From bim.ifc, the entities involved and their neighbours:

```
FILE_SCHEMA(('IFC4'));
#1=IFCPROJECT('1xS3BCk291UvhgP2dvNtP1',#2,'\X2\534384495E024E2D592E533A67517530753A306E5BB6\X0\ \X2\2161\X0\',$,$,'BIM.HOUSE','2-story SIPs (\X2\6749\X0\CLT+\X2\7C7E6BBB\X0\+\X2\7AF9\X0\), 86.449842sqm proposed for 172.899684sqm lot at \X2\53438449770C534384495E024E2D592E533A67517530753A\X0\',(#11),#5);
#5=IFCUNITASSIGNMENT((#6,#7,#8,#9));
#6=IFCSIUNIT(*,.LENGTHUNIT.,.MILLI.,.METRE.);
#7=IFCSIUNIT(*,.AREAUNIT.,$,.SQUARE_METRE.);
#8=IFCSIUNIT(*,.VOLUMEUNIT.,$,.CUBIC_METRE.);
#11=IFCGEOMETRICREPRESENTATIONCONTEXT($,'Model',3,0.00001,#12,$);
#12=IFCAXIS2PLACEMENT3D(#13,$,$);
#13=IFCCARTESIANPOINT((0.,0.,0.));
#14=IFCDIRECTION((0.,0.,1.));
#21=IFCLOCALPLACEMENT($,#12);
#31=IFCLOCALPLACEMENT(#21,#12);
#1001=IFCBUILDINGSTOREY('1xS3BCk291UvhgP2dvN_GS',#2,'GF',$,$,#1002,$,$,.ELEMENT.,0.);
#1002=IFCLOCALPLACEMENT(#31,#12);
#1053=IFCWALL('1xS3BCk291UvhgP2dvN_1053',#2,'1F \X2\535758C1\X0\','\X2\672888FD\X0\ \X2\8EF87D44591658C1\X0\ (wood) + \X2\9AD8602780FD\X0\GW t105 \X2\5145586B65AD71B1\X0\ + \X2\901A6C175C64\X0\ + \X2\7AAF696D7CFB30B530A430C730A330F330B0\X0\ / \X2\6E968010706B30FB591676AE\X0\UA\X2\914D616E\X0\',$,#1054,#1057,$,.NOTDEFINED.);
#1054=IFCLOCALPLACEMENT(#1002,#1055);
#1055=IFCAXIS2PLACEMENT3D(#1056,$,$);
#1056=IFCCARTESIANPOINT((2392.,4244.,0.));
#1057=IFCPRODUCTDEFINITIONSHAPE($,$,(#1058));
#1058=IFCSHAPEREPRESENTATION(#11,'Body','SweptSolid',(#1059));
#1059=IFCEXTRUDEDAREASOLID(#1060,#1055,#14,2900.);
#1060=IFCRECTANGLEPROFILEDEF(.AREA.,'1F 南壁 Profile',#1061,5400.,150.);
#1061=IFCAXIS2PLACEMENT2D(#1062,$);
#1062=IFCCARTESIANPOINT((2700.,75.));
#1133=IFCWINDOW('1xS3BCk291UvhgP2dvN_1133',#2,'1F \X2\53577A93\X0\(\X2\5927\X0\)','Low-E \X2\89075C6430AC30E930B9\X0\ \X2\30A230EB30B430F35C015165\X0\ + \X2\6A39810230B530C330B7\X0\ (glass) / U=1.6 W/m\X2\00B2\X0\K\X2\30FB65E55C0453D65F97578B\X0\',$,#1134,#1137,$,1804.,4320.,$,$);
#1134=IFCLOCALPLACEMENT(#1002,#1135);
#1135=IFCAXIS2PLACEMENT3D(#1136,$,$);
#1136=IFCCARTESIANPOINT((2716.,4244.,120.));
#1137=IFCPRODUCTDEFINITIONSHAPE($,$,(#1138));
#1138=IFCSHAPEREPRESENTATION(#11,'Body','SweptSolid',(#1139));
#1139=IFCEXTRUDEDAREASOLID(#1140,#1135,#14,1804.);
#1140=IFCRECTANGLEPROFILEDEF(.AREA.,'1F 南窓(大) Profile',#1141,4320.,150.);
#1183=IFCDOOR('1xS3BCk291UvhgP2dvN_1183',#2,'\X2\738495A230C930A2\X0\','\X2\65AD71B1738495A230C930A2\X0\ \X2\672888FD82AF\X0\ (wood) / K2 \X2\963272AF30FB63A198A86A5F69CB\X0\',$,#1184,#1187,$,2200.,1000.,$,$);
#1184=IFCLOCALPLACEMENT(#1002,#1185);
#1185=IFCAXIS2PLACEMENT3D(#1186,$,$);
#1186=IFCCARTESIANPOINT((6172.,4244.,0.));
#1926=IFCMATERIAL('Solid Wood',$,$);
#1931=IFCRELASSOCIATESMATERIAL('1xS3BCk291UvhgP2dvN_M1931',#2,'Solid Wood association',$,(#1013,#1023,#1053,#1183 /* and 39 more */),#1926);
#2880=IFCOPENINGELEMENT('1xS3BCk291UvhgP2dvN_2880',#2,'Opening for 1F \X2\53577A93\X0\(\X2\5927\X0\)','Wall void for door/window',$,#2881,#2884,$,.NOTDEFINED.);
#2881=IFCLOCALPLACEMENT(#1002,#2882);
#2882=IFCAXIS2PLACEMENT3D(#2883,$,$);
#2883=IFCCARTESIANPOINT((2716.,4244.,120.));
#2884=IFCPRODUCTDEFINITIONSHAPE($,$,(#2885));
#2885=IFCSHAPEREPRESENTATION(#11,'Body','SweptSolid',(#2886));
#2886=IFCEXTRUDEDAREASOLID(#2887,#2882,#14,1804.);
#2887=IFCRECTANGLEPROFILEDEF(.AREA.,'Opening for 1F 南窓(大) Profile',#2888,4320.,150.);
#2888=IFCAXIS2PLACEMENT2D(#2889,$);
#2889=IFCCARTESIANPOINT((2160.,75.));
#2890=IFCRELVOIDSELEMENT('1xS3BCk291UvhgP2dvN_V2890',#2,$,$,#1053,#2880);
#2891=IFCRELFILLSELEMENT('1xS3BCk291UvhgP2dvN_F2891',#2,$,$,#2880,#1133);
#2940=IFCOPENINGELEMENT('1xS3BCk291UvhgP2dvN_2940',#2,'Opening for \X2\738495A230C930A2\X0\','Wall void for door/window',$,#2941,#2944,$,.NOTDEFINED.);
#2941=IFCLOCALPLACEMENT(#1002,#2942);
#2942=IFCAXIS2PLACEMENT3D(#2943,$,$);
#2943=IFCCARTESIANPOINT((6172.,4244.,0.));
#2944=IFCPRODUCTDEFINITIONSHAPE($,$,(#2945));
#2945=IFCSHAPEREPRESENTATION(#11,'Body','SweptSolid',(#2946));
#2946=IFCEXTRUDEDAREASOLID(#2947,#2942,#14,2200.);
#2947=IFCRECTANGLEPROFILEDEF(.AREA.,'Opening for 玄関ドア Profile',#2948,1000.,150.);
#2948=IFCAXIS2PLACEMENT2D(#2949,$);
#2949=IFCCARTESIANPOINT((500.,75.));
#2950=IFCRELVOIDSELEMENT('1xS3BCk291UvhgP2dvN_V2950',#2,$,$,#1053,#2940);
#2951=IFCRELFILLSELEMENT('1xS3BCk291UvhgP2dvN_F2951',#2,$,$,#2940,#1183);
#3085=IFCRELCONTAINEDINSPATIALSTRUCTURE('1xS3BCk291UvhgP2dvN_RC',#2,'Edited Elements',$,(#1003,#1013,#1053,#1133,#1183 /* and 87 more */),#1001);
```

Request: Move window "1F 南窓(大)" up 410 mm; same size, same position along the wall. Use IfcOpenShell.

```python
import numpy as np
import ifcopenshell
import ifcopenshell.api.geometry
import ifcopenshell.util.placement
import ifcopenshell.util.unit

model = ifcopenshell.open("bim.ifc")
unit_scale = ifcopenshell.util.unit.calculate_unit_scale(model)

window = model.by_id(1133)
opening = window.FillsVoids[0].RelatingOpeningElement
dz = 410.0

shift = np.array([0.0, 0.0, dz])
# The window is not placed relative to its opening, so move both.
for product in (opening, window):
    matrix = ifcopenshell.util.placement.get_local_placement(product.ObjectPlacement)
    matrix[:3, 3] += shift
    ifcopenshell.api.geometry.edit_object_placement(model, product=product, matrix=matrix, is_si=False)

print(f"moved by {dz * unit_scale:+.3f} m")

model.write("bim_v2.ifc")
```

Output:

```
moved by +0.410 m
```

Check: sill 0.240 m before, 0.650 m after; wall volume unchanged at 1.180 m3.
